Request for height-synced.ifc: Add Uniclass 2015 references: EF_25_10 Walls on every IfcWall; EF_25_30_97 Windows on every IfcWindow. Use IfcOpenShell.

First a look at what the model holds.

```python
import ifcopenshell

model = ifcopenshell.open("height-synced.ifc")
print(model.schema)
print("classifications:", [c.Name for c in model.by_type("IfcClassification")])
for ifc_class in ("IfcDoor", "IfcRoof", "IfcStair", "IfcWall", "IfcWindow"):
    print(ifc_class, len(model.by_type(ifc_class)))
```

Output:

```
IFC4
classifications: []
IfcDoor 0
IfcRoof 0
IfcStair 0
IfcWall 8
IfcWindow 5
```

```python
import ifcopenshell
import ifcopenshell.api.classification

model = ifcopenshell.open("height-synced.ifc")

system = ifcopenshell.api.classification.add_classification(model, classification="Uniclass 2015")

codes = {
    "IfcWall": ("EF_25_10", "Walls"),
    "IfcWindow": ("EF_25_30_97", "Windows"),
}
for ifc_class, (code, name) in codes.items():
    products = model.by_type(ifc_class)
    ifcopenshell.api.classification.add_reference(
        model, products=products, classification=system, identification=code, name=name
    )
    print(code, len(products))

model.write("height-synced-out.ifc")
```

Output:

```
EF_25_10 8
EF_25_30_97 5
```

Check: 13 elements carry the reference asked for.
